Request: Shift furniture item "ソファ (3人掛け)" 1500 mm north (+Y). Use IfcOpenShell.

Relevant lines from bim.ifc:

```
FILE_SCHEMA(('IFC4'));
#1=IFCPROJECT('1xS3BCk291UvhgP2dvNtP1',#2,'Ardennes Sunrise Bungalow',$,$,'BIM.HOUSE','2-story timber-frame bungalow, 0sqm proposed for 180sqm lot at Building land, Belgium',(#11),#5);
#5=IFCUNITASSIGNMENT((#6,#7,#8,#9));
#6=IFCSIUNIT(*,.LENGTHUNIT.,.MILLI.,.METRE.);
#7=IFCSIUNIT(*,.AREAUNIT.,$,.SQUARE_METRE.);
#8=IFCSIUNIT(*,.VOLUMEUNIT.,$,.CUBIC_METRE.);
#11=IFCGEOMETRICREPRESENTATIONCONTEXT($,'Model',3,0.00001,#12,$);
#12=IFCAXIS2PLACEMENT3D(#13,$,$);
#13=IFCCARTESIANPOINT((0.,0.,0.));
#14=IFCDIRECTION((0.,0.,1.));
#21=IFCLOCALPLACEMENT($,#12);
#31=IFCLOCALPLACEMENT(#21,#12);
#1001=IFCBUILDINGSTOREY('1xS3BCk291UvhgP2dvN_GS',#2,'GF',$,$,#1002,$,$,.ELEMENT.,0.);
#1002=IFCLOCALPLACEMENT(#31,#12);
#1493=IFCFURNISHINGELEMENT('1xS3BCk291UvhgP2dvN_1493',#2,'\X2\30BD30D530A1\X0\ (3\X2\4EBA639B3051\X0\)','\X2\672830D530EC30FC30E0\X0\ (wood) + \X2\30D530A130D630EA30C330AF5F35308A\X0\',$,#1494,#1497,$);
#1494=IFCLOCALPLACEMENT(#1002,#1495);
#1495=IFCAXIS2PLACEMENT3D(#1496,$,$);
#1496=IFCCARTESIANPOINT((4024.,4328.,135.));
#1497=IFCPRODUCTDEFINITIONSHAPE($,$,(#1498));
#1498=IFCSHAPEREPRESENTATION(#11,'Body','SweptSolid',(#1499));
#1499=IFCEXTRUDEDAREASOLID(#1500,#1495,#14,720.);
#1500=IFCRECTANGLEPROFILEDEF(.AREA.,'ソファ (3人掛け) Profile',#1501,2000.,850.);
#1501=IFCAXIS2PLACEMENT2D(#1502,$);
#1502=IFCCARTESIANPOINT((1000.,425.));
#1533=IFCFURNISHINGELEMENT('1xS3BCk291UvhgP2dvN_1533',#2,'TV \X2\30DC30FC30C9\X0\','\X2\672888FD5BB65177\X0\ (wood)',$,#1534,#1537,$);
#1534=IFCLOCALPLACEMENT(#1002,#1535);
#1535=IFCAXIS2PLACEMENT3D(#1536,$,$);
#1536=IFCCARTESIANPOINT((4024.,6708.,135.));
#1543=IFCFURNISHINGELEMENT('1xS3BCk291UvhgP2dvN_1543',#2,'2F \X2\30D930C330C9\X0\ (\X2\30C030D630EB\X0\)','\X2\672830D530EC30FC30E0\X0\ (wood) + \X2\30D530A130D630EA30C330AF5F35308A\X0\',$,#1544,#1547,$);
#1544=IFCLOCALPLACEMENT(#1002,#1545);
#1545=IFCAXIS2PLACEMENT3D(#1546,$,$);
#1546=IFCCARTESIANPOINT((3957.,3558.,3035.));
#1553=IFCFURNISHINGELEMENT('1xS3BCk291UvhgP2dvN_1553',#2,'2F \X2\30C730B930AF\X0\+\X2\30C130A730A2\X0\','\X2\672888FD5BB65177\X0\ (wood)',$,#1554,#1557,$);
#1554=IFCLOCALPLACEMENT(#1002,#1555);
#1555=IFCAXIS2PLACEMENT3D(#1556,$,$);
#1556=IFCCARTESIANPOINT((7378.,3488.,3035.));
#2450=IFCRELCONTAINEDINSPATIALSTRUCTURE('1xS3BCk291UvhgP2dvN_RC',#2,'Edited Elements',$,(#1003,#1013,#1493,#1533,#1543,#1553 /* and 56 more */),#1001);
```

```python
import ifcopenshell
import ifcopenshell.api.geometry
import ifcopenshell.util.placement
import ifcopenshell.util.unit

model = ifcopenshell.open("bim.ifc")
unit_scale = ifcopenshell.util.unit.calculate_unit_scale(model)

item = model.by_id(1493)
matrix = ifcopenshell.util.placement.get_local_placement(item.ObjectPlacement)
matrix[1, 3] += 1.5 / unit_scale
ifcopenshell.api.geometry.edit_object_placement(model, product=item, matrix=matrix, is_si=False)

print(ifcopenshell.util.placement.get_local_placement(item.ObjectPlacement).round(3) + 0.0)

model.write("bim_edited.ifc")
```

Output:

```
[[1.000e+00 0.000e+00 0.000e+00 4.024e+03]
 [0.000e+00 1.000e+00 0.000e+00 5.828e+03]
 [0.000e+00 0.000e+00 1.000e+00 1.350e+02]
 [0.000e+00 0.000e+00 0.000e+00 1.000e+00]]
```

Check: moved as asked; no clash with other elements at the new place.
